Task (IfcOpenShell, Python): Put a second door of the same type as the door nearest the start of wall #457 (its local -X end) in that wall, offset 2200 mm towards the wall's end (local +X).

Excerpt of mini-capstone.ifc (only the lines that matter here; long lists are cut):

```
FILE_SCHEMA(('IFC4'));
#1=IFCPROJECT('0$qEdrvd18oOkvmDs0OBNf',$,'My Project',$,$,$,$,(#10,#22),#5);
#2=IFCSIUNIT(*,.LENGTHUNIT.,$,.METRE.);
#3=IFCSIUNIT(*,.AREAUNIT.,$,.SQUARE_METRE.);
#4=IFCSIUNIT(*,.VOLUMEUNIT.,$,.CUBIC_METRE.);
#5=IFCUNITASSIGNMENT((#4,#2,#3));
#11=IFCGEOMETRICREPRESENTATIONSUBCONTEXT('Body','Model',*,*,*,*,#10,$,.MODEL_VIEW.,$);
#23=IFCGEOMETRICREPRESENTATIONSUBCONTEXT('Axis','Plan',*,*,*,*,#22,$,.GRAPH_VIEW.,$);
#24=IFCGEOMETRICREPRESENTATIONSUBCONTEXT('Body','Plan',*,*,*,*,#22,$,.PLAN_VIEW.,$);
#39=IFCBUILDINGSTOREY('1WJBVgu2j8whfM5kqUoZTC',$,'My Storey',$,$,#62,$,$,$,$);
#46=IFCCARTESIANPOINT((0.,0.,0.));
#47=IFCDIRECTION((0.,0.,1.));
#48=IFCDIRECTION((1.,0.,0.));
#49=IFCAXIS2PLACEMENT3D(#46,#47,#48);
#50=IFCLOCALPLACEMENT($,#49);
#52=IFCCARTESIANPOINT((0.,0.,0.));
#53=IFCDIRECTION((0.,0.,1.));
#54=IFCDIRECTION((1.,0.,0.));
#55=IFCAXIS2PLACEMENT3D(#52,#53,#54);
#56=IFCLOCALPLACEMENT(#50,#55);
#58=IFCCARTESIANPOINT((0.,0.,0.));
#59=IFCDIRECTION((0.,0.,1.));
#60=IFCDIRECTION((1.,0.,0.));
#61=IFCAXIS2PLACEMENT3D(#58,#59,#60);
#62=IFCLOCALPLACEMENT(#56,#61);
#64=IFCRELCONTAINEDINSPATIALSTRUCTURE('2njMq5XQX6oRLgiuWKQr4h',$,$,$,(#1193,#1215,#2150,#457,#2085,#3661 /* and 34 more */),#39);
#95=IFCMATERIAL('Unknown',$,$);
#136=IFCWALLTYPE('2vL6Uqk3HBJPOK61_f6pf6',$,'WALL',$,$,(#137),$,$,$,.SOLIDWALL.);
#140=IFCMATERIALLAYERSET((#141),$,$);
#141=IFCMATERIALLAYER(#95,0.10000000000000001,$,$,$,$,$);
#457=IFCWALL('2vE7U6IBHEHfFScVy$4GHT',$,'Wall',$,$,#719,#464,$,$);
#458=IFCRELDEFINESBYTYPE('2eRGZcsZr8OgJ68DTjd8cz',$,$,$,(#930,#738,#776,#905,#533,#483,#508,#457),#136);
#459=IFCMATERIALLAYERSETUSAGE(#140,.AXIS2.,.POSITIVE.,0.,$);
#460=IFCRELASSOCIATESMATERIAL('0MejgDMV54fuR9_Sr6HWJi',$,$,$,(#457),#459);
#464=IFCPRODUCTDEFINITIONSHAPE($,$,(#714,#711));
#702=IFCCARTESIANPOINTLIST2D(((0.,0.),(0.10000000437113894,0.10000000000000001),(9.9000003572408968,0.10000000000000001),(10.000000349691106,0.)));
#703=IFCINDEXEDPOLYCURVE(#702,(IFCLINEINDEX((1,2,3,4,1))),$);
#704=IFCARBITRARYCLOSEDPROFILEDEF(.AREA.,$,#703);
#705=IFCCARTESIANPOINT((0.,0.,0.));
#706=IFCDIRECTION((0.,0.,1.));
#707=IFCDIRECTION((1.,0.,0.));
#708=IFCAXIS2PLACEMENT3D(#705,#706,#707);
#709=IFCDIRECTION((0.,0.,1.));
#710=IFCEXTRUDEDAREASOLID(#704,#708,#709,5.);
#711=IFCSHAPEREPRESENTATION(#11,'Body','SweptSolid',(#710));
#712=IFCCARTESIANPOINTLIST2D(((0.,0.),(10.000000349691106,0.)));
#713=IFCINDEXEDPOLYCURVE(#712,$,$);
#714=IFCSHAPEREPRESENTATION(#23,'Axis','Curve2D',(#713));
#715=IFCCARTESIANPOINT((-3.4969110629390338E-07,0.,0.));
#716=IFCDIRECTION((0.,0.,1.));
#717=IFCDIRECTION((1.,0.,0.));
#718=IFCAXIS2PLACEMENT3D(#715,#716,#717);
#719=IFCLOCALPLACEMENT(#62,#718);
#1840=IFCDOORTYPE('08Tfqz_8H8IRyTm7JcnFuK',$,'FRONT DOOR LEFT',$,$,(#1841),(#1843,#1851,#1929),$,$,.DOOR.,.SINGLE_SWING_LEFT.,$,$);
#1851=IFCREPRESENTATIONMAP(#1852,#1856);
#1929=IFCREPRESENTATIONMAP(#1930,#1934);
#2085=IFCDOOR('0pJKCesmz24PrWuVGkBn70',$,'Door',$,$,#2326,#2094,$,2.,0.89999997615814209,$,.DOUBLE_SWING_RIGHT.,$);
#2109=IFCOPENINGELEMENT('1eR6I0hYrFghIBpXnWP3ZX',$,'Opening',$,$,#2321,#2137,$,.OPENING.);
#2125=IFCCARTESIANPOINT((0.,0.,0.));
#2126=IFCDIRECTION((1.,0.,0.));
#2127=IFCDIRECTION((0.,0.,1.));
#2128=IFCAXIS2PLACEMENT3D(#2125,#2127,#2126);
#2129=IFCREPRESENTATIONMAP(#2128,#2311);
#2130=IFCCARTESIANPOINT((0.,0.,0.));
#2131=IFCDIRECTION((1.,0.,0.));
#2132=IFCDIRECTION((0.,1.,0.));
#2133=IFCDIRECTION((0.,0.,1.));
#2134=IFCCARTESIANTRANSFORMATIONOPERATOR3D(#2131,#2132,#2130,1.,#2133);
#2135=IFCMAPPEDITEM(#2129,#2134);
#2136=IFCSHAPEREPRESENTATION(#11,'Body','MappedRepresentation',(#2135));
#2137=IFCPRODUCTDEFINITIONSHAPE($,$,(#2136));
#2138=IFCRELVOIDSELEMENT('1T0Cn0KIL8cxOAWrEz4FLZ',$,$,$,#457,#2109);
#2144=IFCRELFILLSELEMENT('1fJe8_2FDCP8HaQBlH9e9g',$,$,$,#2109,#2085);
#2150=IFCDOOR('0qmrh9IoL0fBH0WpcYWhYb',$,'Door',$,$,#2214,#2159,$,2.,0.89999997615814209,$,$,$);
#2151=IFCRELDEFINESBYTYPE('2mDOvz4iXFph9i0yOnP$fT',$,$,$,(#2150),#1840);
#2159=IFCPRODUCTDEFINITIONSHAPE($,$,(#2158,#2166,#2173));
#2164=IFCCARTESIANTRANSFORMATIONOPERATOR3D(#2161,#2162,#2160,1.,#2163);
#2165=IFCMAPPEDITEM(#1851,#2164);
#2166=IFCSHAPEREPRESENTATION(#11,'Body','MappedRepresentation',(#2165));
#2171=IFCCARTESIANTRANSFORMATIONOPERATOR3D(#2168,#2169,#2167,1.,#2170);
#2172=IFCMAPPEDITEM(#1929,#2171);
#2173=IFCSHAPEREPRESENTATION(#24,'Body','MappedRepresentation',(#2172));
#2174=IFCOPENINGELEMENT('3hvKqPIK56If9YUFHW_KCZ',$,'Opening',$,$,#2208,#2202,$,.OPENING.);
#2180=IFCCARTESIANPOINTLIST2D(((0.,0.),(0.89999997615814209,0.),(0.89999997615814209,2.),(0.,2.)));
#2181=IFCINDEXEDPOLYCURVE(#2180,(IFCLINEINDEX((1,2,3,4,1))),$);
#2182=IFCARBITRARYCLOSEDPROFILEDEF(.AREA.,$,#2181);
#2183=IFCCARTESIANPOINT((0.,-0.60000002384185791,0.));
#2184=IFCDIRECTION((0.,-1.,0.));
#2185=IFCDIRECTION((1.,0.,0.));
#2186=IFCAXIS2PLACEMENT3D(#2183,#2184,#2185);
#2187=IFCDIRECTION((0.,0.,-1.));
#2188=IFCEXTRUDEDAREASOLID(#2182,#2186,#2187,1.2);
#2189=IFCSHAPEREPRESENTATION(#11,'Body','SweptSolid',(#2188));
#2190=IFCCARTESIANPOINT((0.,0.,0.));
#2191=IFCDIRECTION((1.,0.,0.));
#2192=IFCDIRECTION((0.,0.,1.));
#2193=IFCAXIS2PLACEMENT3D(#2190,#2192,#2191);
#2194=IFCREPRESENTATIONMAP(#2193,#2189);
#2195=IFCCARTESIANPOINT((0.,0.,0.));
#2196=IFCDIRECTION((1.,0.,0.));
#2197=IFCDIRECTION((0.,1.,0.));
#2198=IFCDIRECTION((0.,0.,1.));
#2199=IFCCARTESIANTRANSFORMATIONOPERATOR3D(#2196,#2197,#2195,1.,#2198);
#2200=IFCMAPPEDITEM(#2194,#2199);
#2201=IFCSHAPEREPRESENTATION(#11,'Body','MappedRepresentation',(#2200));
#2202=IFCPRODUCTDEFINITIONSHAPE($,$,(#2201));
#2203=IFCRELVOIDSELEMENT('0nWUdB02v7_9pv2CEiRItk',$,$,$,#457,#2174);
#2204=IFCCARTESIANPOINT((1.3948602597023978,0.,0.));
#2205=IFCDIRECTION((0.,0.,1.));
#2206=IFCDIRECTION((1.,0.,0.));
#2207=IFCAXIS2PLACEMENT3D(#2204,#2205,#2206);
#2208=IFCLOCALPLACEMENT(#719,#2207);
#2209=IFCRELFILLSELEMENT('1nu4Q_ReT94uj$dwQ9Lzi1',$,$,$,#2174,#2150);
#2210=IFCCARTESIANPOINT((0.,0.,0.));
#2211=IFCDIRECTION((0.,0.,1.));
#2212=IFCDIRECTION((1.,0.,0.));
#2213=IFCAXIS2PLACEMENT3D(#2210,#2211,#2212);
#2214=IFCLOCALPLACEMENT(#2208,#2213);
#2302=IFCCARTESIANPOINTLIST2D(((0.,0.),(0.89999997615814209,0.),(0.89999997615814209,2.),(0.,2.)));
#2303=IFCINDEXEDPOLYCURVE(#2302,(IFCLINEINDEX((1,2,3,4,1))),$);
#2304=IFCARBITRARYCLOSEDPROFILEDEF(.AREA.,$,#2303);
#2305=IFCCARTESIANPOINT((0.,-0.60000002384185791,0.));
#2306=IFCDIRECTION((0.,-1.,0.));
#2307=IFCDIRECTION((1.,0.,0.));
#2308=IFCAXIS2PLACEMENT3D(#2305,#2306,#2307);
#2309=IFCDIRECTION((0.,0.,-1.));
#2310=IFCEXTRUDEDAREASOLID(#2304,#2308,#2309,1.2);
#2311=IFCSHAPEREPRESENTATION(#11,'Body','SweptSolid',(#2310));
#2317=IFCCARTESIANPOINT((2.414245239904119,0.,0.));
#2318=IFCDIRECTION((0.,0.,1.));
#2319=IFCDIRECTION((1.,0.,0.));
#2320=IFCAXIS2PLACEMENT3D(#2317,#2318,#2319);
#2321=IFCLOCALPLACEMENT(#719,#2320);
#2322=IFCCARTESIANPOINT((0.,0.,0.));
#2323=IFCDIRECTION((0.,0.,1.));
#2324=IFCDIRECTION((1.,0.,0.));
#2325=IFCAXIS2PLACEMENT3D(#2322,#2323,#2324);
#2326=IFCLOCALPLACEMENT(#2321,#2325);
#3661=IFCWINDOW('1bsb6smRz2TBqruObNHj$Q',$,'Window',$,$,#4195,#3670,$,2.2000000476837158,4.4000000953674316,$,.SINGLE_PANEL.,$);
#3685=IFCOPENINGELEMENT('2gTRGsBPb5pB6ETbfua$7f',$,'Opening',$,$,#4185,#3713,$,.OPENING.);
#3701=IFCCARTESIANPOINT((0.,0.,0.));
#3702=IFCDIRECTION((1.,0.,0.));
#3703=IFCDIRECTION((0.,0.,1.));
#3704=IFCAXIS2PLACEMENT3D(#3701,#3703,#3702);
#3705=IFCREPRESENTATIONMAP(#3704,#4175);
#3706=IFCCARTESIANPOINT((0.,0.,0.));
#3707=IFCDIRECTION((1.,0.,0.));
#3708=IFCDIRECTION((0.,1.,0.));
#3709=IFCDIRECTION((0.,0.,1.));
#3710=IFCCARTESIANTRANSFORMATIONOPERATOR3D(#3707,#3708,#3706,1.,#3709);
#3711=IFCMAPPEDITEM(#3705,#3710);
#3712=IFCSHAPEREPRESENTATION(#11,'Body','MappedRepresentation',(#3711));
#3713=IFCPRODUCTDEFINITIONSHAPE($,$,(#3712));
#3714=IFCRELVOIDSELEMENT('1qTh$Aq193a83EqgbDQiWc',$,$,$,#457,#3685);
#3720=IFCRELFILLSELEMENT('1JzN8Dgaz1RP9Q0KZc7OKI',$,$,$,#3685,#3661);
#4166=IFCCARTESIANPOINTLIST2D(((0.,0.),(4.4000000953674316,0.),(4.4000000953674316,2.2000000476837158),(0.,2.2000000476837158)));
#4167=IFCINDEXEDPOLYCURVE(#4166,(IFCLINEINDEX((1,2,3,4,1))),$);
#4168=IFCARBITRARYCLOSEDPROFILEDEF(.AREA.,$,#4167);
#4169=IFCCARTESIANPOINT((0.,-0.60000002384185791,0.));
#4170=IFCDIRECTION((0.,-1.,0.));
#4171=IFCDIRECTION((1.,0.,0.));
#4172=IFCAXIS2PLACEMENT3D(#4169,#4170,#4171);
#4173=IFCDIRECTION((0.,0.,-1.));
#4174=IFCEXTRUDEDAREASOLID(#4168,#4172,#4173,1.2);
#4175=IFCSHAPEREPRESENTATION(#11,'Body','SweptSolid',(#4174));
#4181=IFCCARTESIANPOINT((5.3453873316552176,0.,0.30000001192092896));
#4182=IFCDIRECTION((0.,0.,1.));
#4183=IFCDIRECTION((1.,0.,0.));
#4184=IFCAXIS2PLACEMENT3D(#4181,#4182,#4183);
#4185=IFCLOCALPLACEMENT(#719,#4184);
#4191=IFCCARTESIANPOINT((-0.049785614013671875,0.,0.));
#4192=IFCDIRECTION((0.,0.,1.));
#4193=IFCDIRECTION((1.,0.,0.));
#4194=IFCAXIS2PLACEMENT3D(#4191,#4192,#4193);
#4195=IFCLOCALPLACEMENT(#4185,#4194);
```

```python
import ifcopenshell
import ifcopenshell.api.feature
import ifcopenshell.api.geometry
import ifcopenshell.api.root
import ifcopenshell.geom
import ifcopenshell.util.element
import ifcopenshell.util.placement
import ifcopenshell.util.shape
import ifcopenshell.util.unit

model = ifcopenshell.open("mini-capstone.ifc")
unit_scale = ifcopenshell.util.unit.calculate_unit_scale(model)
settings = ifcopenshell.geom.settings()


def volume(element):
    """Net volume in cubic metres, openings subtracted."""
    shape = ifcopenshell.geom.create_shape(settings, element)
    return ifcopenshell.util.shape.get_volume(shape.geometry)


door = model.by_guid("0qmrh9IoL0fBH0WpcYWhYb")
opening = door.FillsVoids[0].RelatingOpeningElement
wall = opening.VoidsElements[0].RelatingBuildingElement
before = volume(wall)
shift = ifcopenshell.util.placement.get_local_placement(wall.ObjectPlacement)[:3, 0] * 2.2 / unit_scale

# copy_class copies the void relationship, type, container and properties, but no geometry.
new_opening = ifcopenshell.api.root.copy_class(model, product=opening)
new_opening.Representation = ifcopenshell.util.element.copy_deep(
    model, opening.Representation, exclude=["IfcGeometricRepresentationContext", "IfcRepresentationMap"]
)
new_door = ifcopenshell.api.root.copy_class(model, product=door)
new_door.Representation = ifcopenshell.util.element.copy_deep(
    model, door.Representation, exclude=["IfcGeometricRepresentationContext", "IfcRepresentationMap"]
)
ifcopenshell.api.feature.add_filling(model, opening=new_opening, element=new_door)

for old, new in ((opening, new_opening), (door, new_door)):
    matrix = ifcopenshell.util.placement.get_local_placement(old.ObjectPlacement)
    matrix[:3, 3] += shift
    ifcopenshell.api.geometry.edit_object_placement(model, product=new, matrix=matrix, is_si=False)

after = volume(wall)

print(f"wall volume {before:.3f} -> {after:.3f} m3")

model.write("mini-capstone-out.ifc")
```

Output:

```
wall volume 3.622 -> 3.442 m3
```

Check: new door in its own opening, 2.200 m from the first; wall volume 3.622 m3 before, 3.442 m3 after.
